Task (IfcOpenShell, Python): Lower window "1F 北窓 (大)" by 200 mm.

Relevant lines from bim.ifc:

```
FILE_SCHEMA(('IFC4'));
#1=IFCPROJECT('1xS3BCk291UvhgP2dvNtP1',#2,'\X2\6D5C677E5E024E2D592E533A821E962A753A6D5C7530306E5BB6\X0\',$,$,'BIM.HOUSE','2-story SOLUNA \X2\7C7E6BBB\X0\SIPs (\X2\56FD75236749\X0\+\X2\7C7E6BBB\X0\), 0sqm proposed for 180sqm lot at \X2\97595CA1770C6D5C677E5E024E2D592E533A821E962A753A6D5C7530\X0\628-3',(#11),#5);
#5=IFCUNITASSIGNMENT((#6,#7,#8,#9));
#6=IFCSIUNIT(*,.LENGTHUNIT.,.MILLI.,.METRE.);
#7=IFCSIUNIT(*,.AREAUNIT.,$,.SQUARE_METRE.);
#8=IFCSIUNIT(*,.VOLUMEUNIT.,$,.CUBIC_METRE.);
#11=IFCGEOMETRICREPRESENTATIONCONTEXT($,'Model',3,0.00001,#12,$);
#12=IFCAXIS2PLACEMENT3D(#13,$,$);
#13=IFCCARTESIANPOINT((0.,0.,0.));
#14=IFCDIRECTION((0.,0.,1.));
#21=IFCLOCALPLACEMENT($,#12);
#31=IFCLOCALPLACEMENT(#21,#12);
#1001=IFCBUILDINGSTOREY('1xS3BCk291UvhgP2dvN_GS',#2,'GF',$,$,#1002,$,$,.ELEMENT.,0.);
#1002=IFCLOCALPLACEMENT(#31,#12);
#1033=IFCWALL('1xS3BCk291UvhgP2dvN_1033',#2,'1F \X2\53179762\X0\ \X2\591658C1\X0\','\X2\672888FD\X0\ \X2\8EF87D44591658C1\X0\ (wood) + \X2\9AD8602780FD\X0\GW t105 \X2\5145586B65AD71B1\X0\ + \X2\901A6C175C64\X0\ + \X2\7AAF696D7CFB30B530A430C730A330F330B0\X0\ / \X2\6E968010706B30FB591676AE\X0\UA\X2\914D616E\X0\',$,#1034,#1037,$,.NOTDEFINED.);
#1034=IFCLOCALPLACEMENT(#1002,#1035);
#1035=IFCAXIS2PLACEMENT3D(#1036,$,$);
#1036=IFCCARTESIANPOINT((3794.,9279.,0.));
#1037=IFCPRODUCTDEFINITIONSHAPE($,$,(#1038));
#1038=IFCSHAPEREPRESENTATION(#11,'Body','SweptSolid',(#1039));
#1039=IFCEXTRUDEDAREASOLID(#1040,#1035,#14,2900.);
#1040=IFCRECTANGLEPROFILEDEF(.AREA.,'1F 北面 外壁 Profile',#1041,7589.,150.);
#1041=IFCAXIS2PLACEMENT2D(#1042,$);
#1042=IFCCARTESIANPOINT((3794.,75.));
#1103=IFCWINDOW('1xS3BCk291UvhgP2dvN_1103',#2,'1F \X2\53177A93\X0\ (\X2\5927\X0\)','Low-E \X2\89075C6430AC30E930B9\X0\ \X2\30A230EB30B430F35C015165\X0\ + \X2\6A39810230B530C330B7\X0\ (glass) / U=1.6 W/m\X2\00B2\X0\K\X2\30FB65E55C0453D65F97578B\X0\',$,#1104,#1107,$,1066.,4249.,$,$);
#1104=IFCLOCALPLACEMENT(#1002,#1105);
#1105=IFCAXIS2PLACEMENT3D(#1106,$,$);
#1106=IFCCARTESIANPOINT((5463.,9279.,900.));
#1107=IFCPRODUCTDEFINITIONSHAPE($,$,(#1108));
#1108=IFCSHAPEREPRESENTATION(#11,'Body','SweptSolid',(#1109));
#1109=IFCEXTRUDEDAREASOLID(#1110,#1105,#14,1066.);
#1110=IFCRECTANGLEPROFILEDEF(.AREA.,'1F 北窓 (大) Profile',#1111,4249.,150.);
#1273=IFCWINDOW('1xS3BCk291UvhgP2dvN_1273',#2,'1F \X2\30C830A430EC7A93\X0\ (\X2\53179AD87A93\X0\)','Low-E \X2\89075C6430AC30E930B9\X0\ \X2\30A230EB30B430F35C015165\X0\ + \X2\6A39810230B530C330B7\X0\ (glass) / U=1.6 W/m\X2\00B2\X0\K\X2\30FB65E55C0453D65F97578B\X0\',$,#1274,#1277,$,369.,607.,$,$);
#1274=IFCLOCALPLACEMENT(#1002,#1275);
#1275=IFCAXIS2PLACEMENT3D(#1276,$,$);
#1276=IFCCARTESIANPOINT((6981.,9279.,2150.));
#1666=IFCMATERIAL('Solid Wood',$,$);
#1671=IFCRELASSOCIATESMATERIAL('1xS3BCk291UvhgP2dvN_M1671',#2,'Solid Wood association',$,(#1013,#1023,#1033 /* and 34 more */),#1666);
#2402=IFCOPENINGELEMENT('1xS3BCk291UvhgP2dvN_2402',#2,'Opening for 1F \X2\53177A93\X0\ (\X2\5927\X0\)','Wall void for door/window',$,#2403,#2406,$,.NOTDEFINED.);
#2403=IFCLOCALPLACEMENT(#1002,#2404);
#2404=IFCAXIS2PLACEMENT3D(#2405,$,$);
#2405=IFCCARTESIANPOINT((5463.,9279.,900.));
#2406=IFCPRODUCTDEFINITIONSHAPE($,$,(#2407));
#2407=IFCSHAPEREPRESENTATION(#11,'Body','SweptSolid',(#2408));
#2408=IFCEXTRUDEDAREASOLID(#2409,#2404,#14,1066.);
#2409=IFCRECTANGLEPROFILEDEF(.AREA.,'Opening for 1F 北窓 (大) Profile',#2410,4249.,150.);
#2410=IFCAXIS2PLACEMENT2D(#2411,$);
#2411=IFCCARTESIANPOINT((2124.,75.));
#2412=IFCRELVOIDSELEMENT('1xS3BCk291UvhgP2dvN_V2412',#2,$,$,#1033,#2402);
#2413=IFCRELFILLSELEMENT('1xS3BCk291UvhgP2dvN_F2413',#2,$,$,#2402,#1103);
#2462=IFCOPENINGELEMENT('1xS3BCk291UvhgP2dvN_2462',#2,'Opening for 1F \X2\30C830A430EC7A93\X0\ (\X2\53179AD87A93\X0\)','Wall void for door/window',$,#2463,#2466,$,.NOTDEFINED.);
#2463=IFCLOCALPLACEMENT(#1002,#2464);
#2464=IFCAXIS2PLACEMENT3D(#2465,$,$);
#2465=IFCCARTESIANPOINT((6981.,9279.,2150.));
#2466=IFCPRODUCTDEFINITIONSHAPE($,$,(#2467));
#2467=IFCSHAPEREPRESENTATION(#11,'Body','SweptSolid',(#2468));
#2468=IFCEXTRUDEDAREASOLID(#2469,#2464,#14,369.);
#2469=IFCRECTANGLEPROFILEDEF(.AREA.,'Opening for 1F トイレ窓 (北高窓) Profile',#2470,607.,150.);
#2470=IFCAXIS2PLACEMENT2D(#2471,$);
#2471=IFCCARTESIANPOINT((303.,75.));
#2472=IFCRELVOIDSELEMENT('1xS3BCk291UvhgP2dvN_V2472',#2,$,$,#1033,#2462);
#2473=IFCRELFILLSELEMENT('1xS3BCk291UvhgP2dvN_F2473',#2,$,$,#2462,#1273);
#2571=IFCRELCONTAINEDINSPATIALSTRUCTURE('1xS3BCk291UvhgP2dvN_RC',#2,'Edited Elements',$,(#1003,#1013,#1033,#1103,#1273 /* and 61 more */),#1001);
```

```python
import numpy as np
import ifcopenshell
import ifcopenshell.api.geometry
import ifcopenshell.util.placement
import ifcopenshell.util.unit

model = ifcopenshell.open("bim.ifc")
unit_scale = ifcopenshell.util.unit.calculate_unit_scale(model)

window = model.by_guid("1xS3BCk291UvhgP2dvN_1103")
opening = window.FillsVoids[0].RelatingOpeningElement
dz = -0.2 / unit_scale

shift = np.array([0.0, 0.0, dz])
# The window is not placed relative to its opening, so move both.
for product in (opening, window):
    matrix = ifcopenshell.util.placement.get_local_placement(product.ObjectPlacement)
    matrix[:3, 3] += shift
    ifcopenshell.api.geometry.edit_object_placement(model, product=product, matrix=matrix, is_si=False)

print(f"moved by {dz * unit_scale:+.3f} m")

model.write("bim_v2.ifc")
```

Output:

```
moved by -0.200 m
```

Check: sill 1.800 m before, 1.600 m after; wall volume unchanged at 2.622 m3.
